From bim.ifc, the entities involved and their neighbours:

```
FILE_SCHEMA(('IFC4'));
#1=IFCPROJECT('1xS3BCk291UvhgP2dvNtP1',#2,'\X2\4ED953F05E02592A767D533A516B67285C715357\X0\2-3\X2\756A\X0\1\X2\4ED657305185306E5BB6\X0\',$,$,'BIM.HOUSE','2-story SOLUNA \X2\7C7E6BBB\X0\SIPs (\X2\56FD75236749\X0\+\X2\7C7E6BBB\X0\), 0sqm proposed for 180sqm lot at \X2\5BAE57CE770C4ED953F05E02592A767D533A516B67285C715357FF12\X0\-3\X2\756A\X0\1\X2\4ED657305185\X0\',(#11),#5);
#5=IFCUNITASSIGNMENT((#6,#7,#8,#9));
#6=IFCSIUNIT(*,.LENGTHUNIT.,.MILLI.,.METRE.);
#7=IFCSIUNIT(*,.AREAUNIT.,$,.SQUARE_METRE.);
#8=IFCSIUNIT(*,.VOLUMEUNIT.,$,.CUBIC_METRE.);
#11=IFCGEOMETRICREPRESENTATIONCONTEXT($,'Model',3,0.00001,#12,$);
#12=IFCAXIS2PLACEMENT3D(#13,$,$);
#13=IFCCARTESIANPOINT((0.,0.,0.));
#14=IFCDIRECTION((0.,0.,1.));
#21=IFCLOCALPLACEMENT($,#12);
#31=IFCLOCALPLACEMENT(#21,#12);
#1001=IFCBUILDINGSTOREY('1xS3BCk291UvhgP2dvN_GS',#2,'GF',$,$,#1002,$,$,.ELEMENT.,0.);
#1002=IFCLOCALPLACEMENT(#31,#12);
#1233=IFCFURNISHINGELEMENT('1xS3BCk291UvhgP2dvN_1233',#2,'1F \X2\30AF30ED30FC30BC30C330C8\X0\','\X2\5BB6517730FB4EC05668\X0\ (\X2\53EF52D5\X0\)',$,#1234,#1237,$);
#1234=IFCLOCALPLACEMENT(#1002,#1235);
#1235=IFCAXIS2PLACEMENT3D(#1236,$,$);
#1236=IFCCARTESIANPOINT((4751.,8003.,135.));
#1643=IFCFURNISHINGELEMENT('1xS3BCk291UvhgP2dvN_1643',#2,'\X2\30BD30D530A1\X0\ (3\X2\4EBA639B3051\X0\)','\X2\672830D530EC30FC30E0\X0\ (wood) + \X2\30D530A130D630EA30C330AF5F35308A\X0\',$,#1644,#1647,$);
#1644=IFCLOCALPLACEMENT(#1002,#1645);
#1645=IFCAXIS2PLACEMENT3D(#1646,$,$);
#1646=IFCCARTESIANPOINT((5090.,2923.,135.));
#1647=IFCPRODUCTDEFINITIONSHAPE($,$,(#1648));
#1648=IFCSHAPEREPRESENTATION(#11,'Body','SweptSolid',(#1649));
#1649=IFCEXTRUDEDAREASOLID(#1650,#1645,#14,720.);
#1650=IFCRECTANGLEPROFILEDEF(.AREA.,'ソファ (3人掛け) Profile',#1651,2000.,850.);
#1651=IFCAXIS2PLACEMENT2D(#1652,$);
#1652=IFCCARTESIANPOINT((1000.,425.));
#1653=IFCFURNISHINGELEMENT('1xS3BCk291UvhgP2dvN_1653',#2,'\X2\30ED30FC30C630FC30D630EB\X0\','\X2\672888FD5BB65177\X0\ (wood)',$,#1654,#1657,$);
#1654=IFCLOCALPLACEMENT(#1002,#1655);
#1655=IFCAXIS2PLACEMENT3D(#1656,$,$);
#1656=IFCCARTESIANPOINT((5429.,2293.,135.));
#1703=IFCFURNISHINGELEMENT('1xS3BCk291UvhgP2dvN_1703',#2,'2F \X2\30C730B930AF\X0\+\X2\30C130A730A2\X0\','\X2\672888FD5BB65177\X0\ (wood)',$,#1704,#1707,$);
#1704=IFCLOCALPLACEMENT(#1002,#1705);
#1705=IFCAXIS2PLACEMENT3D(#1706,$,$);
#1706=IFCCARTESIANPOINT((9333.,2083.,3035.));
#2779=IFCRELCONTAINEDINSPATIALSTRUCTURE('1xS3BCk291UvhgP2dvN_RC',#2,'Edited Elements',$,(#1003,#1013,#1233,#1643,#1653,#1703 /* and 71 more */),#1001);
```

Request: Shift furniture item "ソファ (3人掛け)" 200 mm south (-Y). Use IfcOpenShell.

```python
import ifcopenshell
import ifcopenshell.api.geometry
import ifcopenshell.util.placement
import ifcopenshell.util.unit

model = ifcopenshell.open("bim.ifc")
unit_scale = ifcopenshell.util.unit.calculate_unit_scale(model)

item = model.by_guid("1xS3BCk291UvhgP2dvN_1643")
matrix = ifcopenshell.util.placement.get_local_placement(item.ObjectPlacement)
matrix[1, 3] -= 0.2 / unit_scale
ifcopenshell.api.geometry.edit_object_placement(model, product=item, matrix=matrix, is_si=False)

print(ifcopenshell.util.placement.get_local_placement(item.ObjectPlacement).round(3) + 0.0)

model.write("bim-out.ifc")
```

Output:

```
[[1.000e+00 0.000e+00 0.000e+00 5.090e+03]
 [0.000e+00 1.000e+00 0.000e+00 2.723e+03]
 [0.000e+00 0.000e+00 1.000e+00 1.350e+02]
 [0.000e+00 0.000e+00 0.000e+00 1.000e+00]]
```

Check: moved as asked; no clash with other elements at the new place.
